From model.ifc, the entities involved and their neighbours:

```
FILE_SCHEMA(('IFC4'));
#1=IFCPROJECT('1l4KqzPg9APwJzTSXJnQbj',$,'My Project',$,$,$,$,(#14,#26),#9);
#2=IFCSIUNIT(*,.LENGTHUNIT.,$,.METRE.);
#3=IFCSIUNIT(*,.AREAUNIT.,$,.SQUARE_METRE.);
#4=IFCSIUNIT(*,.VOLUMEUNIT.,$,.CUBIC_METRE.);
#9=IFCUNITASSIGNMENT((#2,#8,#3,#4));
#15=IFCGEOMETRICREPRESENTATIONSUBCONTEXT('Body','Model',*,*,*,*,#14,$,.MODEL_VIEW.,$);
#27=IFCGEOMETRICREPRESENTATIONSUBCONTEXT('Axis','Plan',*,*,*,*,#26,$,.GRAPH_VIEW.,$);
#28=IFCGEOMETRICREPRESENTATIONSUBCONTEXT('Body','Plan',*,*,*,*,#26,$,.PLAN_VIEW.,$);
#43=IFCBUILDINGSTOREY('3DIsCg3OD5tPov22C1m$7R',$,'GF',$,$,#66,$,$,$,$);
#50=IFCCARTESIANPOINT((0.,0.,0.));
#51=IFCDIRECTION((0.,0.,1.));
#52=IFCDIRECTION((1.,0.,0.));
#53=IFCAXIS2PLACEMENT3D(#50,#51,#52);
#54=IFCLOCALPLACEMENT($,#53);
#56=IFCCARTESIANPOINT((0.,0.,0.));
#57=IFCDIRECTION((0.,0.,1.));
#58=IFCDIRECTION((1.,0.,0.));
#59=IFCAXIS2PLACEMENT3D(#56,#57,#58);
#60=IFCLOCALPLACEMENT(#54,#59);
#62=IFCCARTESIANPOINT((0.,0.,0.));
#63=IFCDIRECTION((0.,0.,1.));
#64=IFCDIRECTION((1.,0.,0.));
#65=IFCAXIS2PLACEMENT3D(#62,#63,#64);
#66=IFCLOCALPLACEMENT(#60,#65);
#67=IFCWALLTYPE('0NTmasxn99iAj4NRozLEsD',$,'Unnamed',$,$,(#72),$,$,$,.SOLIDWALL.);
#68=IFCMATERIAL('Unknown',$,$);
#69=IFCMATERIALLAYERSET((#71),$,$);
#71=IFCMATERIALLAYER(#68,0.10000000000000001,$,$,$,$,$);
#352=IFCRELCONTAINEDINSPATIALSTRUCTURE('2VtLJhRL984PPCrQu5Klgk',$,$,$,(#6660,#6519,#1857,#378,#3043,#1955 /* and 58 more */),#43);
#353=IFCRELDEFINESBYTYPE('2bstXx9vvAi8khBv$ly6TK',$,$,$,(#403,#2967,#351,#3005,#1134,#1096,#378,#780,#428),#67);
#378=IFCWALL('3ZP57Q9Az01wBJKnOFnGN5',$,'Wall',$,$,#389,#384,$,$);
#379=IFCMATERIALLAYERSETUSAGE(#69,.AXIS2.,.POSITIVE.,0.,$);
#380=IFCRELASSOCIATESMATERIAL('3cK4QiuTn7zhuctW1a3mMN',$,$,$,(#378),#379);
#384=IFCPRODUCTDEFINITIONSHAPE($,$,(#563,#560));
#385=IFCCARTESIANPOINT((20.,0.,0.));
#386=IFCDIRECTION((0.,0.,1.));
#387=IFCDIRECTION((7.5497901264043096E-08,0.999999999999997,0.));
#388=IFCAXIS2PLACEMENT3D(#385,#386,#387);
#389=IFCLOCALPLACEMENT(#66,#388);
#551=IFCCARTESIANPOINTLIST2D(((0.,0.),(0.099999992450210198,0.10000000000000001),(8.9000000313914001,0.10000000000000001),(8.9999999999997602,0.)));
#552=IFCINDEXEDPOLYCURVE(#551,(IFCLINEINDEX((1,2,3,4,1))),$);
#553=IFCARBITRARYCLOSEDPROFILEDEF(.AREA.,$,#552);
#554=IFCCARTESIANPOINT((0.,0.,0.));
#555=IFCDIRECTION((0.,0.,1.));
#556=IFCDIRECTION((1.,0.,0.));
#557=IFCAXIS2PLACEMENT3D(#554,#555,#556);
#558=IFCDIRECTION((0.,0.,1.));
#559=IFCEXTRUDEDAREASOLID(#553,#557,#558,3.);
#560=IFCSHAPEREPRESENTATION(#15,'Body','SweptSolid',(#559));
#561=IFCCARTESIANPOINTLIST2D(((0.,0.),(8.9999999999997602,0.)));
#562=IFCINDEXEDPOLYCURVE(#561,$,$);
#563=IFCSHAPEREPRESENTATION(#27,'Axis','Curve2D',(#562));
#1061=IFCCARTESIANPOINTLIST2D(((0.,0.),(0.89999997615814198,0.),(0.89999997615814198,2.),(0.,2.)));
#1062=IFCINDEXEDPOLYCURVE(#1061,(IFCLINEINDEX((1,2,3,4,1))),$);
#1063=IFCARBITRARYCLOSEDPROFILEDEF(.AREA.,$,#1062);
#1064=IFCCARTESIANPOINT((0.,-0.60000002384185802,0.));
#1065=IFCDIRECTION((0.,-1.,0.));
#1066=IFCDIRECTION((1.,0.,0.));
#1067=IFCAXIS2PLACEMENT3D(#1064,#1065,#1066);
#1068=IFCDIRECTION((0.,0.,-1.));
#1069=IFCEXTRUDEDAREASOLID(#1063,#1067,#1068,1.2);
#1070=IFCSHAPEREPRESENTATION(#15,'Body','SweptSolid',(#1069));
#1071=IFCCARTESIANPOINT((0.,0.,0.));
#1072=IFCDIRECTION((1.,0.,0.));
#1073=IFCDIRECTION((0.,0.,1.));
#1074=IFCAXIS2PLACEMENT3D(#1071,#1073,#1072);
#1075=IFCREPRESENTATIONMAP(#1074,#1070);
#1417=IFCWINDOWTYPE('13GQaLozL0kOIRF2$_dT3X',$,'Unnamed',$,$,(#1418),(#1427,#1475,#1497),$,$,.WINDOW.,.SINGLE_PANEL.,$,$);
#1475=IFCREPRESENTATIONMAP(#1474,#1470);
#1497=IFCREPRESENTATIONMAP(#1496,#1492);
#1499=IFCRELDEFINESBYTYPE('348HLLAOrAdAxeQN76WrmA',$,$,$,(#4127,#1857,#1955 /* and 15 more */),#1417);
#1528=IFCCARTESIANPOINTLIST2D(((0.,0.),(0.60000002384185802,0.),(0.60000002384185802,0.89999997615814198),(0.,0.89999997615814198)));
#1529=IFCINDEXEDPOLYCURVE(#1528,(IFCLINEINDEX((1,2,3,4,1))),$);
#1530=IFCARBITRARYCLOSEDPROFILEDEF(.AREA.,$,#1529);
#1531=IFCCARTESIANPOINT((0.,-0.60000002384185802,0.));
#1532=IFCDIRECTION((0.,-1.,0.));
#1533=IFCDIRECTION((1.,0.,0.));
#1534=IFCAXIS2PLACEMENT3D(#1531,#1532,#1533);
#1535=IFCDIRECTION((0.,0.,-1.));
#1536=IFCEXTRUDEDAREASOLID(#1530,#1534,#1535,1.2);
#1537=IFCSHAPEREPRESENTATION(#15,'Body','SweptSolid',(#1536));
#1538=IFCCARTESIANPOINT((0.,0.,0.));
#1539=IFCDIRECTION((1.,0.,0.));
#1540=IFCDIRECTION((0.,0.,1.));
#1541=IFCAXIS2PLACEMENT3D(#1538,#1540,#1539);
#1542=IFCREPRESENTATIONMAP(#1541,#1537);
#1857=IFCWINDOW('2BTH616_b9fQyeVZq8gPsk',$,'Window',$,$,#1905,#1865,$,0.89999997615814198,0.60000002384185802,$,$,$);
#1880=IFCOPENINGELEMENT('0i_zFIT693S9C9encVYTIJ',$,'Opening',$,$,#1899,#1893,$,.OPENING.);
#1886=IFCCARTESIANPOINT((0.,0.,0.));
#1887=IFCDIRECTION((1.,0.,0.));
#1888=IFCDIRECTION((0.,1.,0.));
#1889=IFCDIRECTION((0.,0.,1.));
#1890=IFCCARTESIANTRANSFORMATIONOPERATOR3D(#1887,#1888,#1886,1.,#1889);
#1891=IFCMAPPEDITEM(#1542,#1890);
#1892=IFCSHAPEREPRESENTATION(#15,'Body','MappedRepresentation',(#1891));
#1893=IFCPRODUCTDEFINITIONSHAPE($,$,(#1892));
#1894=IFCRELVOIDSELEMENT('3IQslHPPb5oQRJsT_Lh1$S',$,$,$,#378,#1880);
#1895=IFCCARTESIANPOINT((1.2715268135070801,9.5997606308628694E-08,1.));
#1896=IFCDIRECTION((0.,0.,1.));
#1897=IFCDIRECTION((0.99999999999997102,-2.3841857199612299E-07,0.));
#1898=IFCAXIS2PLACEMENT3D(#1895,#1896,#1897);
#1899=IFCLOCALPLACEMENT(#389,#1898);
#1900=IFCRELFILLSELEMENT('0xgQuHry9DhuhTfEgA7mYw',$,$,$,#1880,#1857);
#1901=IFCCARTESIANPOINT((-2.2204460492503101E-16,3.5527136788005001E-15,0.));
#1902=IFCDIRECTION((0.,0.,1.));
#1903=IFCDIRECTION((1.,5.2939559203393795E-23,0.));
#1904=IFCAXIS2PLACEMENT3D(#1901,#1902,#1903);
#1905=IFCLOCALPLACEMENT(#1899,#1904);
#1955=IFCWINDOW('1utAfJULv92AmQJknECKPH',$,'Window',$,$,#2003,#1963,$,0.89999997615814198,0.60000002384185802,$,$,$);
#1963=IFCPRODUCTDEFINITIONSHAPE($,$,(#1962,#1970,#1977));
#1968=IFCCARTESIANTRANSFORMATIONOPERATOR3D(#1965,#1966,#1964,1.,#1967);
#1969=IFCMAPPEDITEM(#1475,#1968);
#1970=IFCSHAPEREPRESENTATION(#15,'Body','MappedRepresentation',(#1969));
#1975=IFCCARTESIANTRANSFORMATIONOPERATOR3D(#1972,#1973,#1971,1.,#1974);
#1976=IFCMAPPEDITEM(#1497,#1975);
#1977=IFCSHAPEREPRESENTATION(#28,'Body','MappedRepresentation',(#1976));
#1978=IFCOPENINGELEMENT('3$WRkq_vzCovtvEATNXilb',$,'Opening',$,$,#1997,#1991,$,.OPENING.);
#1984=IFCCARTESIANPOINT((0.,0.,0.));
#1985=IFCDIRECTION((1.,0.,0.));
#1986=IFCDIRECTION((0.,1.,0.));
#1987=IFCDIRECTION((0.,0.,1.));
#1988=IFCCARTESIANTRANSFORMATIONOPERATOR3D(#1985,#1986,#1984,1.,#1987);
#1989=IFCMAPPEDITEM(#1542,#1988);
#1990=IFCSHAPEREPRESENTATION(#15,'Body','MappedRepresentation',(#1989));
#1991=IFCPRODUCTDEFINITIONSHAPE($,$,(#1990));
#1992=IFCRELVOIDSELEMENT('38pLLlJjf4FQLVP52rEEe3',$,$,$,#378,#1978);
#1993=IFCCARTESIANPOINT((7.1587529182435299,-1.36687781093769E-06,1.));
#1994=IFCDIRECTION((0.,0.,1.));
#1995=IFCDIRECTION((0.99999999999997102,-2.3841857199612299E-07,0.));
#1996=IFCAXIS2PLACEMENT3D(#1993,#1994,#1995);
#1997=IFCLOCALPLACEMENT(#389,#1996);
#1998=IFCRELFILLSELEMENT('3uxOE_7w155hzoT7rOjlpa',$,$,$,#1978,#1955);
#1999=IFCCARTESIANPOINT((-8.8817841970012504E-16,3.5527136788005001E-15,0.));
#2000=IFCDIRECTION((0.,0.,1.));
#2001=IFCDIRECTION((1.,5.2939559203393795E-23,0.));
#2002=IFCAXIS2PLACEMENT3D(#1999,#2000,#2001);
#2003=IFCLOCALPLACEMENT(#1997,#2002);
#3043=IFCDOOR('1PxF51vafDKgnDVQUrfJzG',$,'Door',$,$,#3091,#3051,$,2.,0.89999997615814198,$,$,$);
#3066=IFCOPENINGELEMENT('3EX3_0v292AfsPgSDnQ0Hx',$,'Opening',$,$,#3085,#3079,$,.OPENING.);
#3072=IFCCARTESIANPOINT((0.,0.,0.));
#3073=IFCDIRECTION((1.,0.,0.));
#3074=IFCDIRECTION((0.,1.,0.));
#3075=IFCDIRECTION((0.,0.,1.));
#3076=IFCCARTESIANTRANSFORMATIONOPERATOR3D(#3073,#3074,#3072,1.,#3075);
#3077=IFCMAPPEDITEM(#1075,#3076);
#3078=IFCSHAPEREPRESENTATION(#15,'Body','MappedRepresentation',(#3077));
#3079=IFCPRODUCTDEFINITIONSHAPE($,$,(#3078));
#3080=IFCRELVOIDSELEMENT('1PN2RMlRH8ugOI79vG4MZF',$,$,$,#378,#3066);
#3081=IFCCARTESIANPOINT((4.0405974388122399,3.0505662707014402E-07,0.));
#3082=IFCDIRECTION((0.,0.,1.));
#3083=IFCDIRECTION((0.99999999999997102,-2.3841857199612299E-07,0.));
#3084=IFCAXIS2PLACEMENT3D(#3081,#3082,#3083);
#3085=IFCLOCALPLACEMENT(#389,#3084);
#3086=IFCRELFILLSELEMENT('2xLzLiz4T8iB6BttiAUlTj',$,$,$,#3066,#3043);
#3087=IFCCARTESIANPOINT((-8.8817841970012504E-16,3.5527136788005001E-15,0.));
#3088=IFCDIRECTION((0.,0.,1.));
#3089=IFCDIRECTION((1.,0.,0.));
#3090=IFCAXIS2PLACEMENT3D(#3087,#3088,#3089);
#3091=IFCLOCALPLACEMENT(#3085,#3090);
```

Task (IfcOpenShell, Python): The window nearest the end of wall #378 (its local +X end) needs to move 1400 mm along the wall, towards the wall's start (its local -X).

```python
import ifcopenshell
import ifcopenshell.api.geometry
import ifcopenshell.util.placement

model = ifcopenshell.open("model.ifc")

window = model.by_guid("1utAfJULv92AmQJknECKPH")
opening = window.FillsVoids[0].RelatingOpeningElement
wall = opening.VoidsElements[0].RelatingBuildingElement

wall_matrix = ifcopenshell.util.placement.get_local_placement(wall.ObjectPlacement)
shift = wall_matrix[:3, 0] * -1.4
before = ifcopenshell.util.placement.get_local_placement(window.ObjectPlacement)[:3, 3].copy()

# The window is placed relative to its opening, so it follows when the opening moves.
matrix = ifcopenshell.util.placement.get_local_placement(opening.ObjectPlacement)
matrix[:3, 3] += shift
ifcopenshell.api.geometry.edit_object_placement(
    model, product=opening, matrix=matrix, is_si=False, should_transform_children=True
)

after = ifcopenshell.util.placement.get_local_placement(window.ObjectPlacement)[:3, 3]
print("window moved by", (after - before).round(3) + 0.0)

model.write("model-out.ifc")
```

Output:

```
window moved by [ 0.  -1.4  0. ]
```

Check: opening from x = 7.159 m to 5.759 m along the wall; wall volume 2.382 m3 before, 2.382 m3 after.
